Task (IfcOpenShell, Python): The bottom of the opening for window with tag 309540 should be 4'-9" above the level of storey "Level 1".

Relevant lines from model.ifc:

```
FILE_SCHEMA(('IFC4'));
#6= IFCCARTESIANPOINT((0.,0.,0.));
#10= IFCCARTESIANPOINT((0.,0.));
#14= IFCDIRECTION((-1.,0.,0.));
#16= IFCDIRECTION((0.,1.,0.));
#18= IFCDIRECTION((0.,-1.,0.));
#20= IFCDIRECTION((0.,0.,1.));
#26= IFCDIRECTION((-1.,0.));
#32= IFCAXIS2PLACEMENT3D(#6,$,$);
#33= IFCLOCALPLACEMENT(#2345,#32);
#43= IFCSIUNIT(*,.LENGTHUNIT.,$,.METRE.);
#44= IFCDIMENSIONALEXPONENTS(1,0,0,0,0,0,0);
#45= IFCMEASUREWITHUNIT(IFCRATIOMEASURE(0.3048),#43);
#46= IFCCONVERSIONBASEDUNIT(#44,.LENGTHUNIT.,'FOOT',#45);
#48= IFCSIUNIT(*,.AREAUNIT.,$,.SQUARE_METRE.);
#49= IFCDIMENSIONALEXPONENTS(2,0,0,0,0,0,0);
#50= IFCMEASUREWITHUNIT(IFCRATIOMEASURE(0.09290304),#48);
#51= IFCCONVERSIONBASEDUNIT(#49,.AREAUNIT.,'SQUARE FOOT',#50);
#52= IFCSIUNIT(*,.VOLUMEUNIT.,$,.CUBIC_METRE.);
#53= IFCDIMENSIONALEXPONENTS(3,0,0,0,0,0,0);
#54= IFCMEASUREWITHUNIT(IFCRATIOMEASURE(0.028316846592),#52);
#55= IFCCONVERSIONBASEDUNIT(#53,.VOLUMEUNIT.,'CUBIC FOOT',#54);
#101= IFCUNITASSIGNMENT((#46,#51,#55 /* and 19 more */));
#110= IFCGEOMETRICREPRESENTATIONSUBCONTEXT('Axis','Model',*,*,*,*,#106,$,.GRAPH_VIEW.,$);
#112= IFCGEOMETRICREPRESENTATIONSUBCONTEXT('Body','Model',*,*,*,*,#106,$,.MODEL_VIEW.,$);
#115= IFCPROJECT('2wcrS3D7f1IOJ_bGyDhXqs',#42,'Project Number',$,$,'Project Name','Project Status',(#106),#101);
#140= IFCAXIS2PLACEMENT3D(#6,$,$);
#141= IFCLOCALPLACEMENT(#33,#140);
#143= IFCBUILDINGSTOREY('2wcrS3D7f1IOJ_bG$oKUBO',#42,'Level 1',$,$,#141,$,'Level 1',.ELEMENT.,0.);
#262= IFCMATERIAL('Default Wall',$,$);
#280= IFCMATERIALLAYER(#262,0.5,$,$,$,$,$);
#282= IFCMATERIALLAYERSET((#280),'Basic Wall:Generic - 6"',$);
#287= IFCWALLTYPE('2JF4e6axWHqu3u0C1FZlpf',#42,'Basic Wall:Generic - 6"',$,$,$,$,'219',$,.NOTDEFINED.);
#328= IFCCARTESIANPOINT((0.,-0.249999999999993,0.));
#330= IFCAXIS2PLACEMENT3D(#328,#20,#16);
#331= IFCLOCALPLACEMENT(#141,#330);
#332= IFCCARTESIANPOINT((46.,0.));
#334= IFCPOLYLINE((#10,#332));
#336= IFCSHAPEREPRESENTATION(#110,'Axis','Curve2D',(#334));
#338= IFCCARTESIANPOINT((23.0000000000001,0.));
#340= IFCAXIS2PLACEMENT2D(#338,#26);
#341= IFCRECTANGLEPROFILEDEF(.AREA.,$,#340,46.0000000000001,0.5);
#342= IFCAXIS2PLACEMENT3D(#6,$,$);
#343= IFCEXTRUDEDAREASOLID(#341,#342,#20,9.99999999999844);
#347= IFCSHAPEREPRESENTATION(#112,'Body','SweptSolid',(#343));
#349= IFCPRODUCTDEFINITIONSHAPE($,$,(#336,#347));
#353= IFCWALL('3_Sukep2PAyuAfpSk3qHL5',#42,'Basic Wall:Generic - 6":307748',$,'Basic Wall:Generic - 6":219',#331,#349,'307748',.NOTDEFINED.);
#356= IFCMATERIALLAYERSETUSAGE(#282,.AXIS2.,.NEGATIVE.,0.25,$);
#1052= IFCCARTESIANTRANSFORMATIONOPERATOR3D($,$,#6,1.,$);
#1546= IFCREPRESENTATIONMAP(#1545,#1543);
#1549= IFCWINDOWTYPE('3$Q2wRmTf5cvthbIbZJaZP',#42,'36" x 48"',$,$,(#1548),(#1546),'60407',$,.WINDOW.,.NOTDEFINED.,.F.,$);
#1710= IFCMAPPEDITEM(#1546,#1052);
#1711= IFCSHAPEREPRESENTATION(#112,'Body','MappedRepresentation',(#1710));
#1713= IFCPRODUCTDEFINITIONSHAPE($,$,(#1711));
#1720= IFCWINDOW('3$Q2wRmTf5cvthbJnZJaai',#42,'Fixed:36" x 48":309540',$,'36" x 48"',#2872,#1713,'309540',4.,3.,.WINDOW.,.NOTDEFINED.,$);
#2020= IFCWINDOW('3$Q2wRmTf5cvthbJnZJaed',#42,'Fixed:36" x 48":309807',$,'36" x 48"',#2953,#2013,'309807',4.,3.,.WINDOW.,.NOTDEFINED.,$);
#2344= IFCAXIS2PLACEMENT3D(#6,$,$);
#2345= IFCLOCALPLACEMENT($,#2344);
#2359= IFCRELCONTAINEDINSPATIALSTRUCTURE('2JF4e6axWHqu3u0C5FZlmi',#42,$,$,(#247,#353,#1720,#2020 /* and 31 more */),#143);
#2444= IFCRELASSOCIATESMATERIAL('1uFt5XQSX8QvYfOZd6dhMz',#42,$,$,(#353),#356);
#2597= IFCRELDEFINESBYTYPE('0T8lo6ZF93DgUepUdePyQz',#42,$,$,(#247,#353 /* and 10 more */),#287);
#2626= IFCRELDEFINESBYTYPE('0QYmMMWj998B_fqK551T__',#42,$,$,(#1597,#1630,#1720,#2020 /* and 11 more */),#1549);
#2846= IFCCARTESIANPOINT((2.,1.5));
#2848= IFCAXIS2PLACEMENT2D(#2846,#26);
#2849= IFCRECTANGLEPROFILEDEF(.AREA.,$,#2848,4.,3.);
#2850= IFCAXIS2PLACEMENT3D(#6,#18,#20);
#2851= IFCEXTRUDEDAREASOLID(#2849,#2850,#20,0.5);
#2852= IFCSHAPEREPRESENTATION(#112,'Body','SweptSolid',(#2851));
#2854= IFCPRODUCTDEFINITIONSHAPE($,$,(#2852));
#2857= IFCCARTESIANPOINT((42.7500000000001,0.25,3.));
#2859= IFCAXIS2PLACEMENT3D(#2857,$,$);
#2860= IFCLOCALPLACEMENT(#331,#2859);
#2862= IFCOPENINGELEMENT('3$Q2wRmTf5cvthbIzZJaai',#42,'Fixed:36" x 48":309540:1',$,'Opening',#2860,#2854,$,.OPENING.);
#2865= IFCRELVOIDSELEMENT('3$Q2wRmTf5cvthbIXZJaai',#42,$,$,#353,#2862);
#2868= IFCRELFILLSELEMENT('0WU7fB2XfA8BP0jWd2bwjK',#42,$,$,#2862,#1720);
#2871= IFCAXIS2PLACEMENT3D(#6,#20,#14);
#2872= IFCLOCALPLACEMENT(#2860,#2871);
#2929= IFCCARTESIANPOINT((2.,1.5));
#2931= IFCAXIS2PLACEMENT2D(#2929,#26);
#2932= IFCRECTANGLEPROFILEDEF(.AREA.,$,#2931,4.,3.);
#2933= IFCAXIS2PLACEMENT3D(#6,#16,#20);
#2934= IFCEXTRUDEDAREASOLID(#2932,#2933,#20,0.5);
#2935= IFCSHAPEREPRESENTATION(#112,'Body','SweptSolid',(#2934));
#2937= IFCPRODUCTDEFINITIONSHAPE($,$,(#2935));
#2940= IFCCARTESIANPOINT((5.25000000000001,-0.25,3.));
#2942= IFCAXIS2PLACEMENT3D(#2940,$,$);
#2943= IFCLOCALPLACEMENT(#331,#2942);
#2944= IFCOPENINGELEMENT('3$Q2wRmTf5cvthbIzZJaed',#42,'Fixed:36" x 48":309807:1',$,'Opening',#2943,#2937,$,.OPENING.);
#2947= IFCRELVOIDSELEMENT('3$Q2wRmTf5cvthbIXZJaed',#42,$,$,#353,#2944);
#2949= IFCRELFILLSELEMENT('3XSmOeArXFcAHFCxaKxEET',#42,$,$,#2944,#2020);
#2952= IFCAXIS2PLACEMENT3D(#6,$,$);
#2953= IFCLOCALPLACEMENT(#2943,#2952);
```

```python
import numpy as np
import ifcopenshell
import ifcopenshell.api.geometry
import ifcopenshell.geom
import ifcopenshell.util.element
import ifcopenshell.util.placement
import ifcopenshell.util.shape
import ifcopenshell.util.unit

model = ifcopenshell.open("model.ifc")
unit_scale = ifcopenshell.util.unit.calculate_unit_scale(model)

window = model.by_guid("3$Q2wRmTf5cvthbJnZJaai")
opening = window.FillsVoids[0].RelatingOpeningElement
storey = ifcopenshell.util.element.get_container(window, ifc_class="IfcBuildingStorey")
level = ifcopenshell.util.placement.get_local_placement(storey.ObjectPlacement)[2, 3]

# The opening's origin need not be at the sill, so measure its lowest point.
shape = ifcopenshell.geom.create_shape(ifcopenshell.geom.settings(), opening)
bottom = ifcopenshell.util.shape.get_shape_bottom_elevation(shape, shape.geometry) / unit_scale
dz = level + 57 * 0.0254 / unit_scale - bottom

shift = np.array([0.0, 0.0, dz])
# The window is placed relative to its opening, so it follows when the opening moves.
matrix = ifcopenshell.util.placement.get_local_placement(opening.ObjectPlacement)
matrix[:3, 3] += shift
ifcopenshell.api.geometry.edit_object_placement(
    model, product=opening, matrix=matrix, is_si=False, should_transform_children=True
)

print(f"moved by {dz * unit_scale:+.3f} m")

model.write("model_updated.ifc")
```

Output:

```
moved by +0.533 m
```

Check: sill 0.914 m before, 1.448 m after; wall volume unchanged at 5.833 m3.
